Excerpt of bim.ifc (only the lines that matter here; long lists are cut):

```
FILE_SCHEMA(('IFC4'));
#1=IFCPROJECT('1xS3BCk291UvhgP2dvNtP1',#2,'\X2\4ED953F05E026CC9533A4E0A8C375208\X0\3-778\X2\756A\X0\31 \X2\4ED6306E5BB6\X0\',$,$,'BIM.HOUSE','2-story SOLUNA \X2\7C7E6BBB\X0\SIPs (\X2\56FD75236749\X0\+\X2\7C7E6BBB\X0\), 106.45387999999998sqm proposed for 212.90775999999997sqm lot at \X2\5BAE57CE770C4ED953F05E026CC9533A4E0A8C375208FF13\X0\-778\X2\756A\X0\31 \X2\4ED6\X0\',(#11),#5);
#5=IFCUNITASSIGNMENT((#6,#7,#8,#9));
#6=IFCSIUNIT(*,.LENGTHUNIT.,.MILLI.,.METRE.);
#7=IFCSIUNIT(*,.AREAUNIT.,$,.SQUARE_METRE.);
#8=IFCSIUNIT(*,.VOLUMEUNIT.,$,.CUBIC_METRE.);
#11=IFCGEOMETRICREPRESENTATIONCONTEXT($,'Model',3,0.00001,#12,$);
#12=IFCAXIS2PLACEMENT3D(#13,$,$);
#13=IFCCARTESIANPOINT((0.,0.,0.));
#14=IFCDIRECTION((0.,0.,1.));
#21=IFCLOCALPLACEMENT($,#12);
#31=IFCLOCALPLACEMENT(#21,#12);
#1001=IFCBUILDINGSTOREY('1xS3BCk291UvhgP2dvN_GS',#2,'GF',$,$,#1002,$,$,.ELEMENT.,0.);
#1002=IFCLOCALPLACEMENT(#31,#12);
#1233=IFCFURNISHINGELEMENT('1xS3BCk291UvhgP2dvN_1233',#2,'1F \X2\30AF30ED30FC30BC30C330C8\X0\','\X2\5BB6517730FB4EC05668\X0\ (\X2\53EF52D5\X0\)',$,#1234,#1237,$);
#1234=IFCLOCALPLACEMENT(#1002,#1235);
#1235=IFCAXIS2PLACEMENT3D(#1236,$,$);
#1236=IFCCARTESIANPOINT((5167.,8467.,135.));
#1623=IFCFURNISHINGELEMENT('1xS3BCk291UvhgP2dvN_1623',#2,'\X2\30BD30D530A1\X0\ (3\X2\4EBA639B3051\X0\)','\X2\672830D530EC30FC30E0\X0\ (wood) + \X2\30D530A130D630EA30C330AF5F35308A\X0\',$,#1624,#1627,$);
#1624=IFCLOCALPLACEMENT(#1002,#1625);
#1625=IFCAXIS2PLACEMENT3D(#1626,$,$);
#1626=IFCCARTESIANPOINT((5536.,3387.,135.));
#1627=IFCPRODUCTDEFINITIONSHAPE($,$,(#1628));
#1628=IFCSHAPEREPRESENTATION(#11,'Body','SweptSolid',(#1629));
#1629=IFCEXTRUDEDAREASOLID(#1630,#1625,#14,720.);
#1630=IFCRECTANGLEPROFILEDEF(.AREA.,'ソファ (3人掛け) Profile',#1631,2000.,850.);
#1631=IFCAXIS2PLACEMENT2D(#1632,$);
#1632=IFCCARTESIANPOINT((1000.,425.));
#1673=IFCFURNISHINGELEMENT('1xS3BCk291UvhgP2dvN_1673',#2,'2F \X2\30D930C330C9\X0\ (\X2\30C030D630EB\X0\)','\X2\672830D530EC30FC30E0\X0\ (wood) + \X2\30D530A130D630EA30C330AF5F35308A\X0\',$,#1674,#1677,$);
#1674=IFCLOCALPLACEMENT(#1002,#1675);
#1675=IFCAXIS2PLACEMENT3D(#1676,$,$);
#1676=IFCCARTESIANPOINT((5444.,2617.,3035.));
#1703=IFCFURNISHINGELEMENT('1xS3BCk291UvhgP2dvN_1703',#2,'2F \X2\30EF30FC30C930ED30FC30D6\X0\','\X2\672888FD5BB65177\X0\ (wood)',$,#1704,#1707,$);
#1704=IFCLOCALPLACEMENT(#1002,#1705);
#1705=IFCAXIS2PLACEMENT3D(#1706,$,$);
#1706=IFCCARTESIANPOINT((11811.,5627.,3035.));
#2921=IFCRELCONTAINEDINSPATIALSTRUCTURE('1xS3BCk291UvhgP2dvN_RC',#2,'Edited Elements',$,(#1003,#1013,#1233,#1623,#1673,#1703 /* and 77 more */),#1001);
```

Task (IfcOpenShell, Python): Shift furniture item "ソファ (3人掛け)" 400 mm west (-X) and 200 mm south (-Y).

```python
import ifcopenshell
import ifcopenshell.api.geometry
import ifcopenshell.util.placement
import ifcopenshell.util.unit

model = ifcopenshell.open("bim.ifc")
unit_scale = ifcopenshell.util.unit.calculate_unit_scale(model)

item = model.by_id(1623)
matrix = ifcopenshell.util.placement.get_local_placement(item.ObjectPlacement)
matrix[0, 3] -= 0.4 / unit_scale
matrix[1, 3] -= 0.2 / unit_scale
ifcopenshell.api.geometry.edit_object_placement(model, product=item, matrix=matrix, is_si=False)

print(ifcopenshell.util.placement.get_local_placement(item.ObjectPlacement).round(3) + 0.0)

model.write("bim_updated.ifc")
```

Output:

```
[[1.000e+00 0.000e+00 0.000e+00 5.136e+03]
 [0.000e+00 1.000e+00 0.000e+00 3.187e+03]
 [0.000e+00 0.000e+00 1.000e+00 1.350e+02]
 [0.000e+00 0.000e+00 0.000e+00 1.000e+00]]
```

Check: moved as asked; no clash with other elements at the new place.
